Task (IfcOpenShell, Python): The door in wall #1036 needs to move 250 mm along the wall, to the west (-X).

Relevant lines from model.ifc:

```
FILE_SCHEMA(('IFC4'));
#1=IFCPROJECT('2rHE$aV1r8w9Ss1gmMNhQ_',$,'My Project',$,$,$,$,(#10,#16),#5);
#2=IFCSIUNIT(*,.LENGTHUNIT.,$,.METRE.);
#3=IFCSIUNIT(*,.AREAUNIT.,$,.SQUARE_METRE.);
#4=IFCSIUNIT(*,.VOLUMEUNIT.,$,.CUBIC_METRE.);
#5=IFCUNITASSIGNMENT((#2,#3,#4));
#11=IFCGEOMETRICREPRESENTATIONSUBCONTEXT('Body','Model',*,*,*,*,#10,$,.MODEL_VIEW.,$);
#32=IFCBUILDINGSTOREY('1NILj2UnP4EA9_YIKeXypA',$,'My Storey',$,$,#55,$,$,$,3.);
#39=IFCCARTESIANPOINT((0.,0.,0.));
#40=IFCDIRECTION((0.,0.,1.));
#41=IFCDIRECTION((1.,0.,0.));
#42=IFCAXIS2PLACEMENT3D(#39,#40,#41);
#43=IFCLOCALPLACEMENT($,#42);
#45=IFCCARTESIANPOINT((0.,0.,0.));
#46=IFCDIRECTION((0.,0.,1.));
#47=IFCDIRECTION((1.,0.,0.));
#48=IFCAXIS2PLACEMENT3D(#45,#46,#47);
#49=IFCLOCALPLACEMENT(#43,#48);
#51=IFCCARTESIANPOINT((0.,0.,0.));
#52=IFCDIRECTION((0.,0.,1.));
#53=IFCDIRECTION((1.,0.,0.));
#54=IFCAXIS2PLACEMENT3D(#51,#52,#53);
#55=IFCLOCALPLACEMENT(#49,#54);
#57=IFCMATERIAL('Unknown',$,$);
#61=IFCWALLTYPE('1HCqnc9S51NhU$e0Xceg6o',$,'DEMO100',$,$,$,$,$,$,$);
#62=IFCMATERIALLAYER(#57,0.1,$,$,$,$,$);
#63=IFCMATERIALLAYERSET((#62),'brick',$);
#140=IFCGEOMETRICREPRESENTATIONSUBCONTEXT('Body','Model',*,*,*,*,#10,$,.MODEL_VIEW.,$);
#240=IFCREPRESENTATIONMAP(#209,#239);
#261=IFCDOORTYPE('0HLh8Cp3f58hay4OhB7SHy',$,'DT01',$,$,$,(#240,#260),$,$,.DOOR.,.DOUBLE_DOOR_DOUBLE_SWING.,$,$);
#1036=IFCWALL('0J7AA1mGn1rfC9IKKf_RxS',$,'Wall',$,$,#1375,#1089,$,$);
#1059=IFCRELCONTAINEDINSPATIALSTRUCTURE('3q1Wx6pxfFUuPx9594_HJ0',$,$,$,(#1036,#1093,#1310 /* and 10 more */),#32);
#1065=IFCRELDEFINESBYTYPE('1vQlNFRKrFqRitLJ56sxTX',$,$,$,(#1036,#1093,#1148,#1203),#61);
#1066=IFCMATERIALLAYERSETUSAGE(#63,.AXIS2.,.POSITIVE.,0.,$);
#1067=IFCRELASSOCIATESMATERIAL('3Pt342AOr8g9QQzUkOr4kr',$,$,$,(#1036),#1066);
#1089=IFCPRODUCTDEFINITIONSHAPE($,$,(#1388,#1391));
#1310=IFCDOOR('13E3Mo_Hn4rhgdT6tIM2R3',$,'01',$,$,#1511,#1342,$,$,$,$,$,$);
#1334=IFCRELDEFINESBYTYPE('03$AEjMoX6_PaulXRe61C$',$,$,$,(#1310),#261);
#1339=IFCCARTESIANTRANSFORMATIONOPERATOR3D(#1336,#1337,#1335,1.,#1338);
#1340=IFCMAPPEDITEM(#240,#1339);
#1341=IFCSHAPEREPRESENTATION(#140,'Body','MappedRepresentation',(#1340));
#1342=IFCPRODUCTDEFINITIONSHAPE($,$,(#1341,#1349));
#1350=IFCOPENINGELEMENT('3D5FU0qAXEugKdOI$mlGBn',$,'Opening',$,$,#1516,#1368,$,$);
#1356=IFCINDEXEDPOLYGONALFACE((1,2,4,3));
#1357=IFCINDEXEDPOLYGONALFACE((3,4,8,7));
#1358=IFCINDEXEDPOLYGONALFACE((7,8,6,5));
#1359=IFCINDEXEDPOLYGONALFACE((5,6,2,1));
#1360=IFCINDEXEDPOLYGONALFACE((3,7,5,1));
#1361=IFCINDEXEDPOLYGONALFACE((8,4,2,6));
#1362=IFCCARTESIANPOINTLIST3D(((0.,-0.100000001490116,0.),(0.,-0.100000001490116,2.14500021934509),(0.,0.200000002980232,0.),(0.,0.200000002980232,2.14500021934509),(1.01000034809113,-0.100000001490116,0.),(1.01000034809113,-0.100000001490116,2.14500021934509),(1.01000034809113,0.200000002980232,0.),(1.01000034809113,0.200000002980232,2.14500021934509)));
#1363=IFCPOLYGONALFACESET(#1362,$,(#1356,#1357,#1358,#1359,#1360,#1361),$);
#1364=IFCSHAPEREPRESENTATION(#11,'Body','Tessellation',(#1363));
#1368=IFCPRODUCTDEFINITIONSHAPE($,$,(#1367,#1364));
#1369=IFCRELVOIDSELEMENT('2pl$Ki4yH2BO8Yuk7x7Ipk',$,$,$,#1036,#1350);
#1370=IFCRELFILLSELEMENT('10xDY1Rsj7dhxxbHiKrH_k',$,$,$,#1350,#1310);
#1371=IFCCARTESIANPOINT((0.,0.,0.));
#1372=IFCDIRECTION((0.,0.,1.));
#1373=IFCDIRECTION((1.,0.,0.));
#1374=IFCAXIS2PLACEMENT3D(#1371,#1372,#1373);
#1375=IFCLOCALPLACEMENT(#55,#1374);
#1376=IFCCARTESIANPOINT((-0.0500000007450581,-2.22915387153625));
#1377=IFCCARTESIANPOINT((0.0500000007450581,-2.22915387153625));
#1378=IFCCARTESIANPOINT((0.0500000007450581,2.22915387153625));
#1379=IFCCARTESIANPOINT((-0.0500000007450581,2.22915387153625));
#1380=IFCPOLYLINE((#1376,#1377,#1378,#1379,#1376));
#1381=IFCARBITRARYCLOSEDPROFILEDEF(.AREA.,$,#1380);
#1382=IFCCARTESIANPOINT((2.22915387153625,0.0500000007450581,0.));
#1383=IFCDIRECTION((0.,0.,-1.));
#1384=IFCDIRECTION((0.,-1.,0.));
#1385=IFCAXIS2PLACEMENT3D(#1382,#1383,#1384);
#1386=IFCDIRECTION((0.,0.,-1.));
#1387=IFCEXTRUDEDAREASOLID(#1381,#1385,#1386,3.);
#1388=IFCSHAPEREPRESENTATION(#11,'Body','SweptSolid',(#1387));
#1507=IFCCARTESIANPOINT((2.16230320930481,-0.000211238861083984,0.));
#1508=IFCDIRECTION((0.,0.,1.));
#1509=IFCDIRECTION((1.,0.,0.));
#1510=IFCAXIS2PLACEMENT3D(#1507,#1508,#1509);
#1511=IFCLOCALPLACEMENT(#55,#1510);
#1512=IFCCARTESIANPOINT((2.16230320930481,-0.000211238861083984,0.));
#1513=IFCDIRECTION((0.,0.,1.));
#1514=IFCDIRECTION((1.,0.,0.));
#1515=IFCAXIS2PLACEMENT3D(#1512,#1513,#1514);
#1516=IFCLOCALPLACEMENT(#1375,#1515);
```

```python
import ifcopenshell
import ifcopenshell.api.geometry
import ifcopenshell.util.placement
import ifcopenshell.util.unit

model = ifcopenshell.open("model.ifc")
unit_scale = ifcopenshell.util.unit.calculate_unit_scale(model)

door = model.by_id(1310)
opening = door.FillsVoids[0].RelatingOpeningElement
wall = opening.VoidsElements[0].RelatingBuildingElement

wall_matrix = ifcopenshell.util.placement.get_local_placement(wall.ObjectPlacement)
shift = wall_matrix[:3, 0] * -0.25 / unit_scale
before = ifcopenshell.util.placement.get_local_placement(door.ObjectPlacement)[:3, 3].copy()

# The door is not placed relative to its opening, so move both.
for product in (opening, door):
    matrix = ifcopenshell.util.placement.get_local_placement(product.ObjectPlacement)
    matrix[:3, 3] += shift
    ifcopenshell.api.geometry.edit_object_placement(model, product=product, matrix=matrix, is_si=False)

after = ifcopenshell.util.placement.get_local_placement(door.ObjectPlacement)[:3, 3]
print("door moved by", (after - before).round(3) + 0.0)

model.write("model_updated.ifc")
```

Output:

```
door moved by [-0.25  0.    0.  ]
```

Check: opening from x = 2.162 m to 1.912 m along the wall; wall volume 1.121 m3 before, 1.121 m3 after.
